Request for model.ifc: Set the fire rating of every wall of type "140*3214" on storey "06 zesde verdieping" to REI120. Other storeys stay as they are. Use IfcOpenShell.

First a look at what the model holds.

```python
import ifcopenshell
import ifcopenshell.util.element

model = ifcopenshell.open("model.ifc")
print(model.schema)
storey = next(s for s in model.by_type("IfcBuildingStorey") if s.Name == "06 zesde verdieping")
walls = [e for e in ifcopenshell.util.element.get_decomposition(storey) if e.is_a("IfcWall")]
seen = {}
for e in walls:
    element_type = ifcopenshell.util.element.get_type(e)
    key = (element_type.Name if element_type != e and element_type else None, ifcopenshell.util.element.get_pset(e, "Pset_WallCommon", "FireRating"))
    seen[key] = seen.get(key, 0) + 1
for (name, value), count in sorted(seen.items(), key=str):
    print(count, "x", name, "|", value)
```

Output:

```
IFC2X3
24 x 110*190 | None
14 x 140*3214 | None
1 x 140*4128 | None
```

```python
import ifcopenshell
import ifcopenshell.api.pset
import ifcopenshell.util.element

model = ifcopenshell.open("model.ifc")

storey = next(s for s in model.by_type("IfcBuildingStorey") if s.Name == "06 zesde verdieping")
walls = [e for e in ifcopenshell.util.element.get_decomposition(storey) if e.is_a("IfcWall")]

count = 0
for e in walls:
    element_type = ifcopenshell.util.element.get_type(e)
    if element_type in (None, e) or element_type.Name != "140*3214":
        continue
    found = ifcopenshell.util.element.get_pset(e, "Pset_WallCommon", should_inherit=False)
    if found:
        pset = model.by_id(found["id"])
        if len(ifcopenshell.util.element.get_elements_by_pset(pset)) > 1:
            pset = ifcopenshell.api.pset.unshare_pset(model, products=[e], pset=pset)[0]
    else:
        pset = ifcopenshell.api.pset.add_pset(model, product=e, name="Pset_WallCommon")
    ifcopenshell.api.pset.edit_pset(model, pset=pset, properties={"FireRating": "REI120"})
    count += 1

print(count, "walls updated")

model.write("model_rev.ifc")
```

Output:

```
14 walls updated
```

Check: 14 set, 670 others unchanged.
